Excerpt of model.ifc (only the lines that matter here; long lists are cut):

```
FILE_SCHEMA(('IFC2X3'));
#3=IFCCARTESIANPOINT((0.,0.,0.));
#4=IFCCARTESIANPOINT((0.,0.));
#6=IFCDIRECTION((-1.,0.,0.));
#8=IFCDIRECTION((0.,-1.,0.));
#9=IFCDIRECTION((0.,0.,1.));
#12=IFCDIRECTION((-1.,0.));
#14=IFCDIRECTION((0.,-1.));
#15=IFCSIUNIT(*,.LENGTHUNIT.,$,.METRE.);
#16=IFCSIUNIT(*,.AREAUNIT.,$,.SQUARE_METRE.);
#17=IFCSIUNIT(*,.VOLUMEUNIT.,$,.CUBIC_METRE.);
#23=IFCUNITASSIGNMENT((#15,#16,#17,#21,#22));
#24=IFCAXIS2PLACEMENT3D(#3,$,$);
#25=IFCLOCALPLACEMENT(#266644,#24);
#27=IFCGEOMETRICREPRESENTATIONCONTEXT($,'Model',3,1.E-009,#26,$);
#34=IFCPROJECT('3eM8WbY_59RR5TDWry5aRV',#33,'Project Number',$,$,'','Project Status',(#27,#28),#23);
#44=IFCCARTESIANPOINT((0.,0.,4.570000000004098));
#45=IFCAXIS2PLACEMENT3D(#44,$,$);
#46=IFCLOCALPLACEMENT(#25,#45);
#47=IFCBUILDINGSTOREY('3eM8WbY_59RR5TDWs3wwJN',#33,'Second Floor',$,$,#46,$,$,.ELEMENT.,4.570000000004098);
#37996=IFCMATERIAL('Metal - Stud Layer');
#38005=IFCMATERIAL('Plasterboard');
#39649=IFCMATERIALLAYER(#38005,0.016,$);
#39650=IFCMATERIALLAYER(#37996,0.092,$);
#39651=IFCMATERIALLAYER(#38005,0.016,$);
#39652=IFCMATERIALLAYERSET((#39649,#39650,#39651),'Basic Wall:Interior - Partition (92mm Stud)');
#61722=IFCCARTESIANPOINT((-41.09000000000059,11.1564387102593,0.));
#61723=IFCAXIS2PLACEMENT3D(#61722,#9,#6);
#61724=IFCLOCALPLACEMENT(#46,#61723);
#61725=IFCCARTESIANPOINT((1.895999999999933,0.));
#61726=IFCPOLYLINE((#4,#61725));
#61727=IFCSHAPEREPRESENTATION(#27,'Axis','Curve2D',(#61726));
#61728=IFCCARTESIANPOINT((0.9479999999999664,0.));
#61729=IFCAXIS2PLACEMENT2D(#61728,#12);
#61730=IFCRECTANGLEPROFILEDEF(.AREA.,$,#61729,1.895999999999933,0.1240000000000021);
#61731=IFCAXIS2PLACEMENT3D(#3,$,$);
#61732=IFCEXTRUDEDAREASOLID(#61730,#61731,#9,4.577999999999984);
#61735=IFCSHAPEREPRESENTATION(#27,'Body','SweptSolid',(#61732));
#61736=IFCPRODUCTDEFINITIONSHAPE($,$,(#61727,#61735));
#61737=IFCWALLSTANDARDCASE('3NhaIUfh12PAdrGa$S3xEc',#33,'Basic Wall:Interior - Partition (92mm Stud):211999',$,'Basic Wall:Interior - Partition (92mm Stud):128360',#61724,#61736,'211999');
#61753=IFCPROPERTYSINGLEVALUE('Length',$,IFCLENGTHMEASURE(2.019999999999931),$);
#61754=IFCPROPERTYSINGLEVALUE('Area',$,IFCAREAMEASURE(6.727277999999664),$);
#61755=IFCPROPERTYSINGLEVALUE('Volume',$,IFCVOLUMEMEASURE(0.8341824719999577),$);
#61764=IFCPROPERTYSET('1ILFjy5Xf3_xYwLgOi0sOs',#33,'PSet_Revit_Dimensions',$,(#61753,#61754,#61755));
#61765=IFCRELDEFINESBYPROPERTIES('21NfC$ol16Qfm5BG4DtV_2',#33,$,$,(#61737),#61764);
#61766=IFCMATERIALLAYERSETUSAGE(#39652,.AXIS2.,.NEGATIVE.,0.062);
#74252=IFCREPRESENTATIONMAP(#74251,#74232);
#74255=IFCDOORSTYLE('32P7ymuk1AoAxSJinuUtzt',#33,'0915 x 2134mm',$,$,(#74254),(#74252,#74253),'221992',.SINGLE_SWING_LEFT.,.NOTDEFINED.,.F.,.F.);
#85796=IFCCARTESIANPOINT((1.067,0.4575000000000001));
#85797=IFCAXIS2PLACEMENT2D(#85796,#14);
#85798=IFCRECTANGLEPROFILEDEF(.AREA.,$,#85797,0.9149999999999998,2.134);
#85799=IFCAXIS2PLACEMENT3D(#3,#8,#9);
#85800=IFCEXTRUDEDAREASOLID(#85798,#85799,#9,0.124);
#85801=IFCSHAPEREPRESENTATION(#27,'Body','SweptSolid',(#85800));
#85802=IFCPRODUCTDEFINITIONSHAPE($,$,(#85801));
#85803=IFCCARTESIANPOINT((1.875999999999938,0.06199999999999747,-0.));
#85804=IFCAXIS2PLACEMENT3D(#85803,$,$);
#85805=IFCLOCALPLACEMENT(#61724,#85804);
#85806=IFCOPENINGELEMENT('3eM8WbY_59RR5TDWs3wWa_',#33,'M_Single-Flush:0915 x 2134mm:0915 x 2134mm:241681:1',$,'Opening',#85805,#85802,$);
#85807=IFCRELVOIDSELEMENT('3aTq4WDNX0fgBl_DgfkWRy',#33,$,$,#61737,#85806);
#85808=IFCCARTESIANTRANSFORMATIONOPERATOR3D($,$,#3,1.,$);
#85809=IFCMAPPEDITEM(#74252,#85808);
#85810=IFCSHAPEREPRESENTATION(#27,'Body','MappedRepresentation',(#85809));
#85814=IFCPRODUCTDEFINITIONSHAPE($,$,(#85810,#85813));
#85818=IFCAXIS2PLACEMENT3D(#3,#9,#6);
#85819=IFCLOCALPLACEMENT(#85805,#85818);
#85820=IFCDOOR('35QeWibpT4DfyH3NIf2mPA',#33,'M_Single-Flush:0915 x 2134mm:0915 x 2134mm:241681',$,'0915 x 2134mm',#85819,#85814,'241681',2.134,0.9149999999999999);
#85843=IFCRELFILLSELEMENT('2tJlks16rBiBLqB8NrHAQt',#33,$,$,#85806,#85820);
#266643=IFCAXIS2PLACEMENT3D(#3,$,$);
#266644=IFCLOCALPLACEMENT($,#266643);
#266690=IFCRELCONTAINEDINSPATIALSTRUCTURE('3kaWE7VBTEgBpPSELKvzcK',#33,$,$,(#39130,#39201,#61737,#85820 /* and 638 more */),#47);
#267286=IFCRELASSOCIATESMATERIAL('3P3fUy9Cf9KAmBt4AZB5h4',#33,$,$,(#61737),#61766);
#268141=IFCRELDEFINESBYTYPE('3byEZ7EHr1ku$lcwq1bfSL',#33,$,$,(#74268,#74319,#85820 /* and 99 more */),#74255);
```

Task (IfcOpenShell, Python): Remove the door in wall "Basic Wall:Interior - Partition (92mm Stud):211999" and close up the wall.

```python
import ifcopenshell
import ifcopenshell.api.feature
import ifcopenshell.api.pset
import ifcopenshell.api.root
import ifcopenshell.geom
import ifcopenshell.util.element
import ifcopenshell.util.shape
import ifcopenshell.util.unit

model = ifcopenshell.open("model.ifc")
area_scale = ifcopenshell.util.unit.calculate_unit_scale(model, "AREAUNIT")
volume_scale = ifcopenshell.util.unit.calculate_unit_scale(model, "VOLUMEUNIT")
settings = ifcopenshell.geom.settings()


def volume(element):
    """Net volume in cubic metres, openings subtracted."""
    shape = ifcopenshell.geom.create_shape(settings, element)
    return ifcopenshell.util.shape.get_volume(shape.geometry)


door = model.by_guid("35QeWibpT4DfyH3NIf2mPA")
opening = door.FillsVoids[0].RelatingOpeningElement
wall = opening.VoidsElements[0].RelatingBuildingElement
before = volume(wall)

ifcopenshell.api.root.remove_product(model, product=door)
ifcopenshell.api.feature.remove_feature(model, feature=opening)

after = volume(wall)
thickness = 0.124  # wall thickness in metres

# Update the wall's stored quantities.
pset = model.by_id(ifcopenshell.util.element.get_pset(wall, "PSet_Revit_Dimensions", should_inherit=False)["id"])
ifcopenshell.api.pset.edit_pset(model, pset=pset, properties={
    "Area": model.create_entity("IfcAreaMeasure", after / thickness / area_scale),
    "Volume": model.create_entity("IfcVolumeMeasure", after / volume_scale),
})

print(f"wall volume {before:.3f} -> {after:.3f} m3")

model.write("model_v2.ifc")
```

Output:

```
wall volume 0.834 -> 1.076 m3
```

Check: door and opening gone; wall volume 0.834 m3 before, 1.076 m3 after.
